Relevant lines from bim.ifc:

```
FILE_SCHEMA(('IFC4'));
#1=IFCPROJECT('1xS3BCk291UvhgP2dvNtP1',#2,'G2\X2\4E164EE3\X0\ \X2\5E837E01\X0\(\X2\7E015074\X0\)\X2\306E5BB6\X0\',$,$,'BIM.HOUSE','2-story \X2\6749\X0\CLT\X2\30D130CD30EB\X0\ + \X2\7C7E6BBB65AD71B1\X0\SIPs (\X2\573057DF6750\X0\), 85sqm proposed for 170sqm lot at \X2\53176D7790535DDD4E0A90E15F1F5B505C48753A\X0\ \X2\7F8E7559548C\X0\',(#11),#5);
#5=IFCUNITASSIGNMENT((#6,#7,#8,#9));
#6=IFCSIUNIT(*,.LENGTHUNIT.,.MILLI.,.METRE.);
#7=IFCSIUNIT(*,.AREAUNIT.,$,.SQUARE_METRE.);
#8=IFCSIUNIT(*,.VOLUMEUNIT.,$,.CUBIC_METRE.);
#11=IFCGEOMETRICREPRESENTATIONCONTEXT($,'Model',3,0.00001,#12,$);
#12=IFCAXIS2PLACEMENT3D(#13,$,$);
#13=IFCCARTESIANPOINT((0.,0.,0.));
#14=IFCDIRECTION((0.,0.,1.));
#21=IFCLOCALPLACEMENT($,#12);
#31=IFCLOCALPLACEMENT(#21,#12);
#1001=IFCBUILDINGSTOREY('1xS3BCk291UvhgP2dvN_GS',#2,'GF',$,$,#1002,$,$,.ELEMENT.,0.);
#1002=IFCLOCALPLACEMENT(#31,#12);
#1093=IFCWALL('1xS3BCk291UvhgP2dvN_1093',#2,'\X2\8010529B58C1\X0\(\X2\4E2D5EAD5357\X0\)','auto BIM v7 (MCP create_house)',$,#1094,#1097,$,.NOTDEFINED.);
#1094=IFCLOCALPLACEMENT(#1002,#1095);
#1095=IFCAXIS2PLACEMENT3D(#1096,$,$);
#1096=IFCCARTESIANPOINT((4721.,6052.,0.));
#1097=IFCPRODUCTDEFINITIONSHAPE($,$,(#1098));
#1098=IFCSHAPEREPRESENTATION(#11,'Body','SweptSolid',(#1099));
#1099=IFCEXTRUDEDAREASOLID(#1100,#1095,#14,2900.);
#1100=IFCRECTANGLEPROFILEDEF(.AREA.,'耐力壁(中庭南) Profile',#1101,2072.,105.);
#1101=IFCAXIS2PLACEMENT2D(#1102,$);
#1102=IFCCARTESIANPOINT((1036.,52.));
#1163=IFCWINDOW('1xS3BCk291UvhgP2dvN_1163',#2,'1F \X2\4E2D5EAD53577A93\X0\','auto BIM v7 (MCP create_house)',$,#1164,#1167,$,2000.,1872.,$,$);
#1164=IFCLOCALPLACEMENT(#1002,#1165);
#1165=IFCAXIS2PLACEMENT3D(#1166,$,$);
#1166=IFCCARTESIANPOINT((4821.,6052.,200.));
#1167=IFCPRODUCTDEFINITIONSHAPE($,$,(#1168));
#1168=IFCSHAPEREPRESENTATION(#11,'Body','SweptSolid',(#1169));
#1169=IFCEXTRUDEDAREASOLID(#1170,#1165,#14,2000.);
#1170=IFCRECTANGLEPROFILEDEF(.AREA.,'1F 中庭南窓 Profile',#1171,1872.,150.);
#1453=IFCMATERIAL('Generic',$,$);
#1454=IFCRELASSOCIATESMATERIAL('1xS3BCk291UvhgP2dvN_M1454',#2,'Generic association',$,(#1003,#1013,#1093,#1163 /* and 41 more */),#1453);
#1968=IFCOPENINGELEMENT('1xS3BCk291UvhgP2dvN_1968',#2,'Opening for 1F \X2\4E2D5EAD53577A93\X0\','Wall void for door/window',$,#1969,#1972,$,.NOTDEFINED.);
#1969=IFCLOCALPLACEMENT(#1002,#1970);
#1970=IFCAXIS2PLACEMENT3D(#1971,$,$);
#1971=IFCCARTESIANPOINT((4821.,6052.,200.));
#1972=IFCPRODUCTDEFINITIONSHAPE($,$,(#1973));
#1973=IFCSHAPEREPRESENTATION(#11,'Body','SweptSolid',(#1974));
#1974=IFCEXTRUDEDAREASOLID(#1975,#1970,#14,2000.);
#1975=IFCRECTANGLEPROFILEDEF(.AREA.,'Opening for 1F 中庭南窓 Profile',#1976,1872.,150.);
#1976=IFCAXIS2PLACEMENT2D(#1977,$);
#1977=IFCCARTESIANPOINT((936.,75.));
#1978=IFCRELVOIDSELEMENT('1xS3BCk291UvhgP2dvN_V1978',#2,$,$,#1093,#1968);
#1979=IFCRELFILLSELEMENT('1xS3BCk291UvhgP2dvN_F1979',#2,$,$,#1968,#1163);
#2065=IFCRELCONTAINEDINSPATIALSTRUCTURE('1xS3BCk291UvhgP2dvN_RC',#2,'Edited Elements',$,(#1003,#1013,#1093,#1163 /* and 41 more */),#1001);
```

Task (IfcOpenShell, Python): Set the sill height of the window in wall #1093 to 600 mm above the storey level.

```python
import numpy as np
import ifcopenshell
import ifcopenshell.api.geometry
import ifcopenshell.geom
import ifcopenshell.util.element
import ifcopenshell.util.placement
import ifcopenshell.util.shape
import ifcopenshell.util.unit

model = ifcopenshell.open("bim.ifc")
unit_scale = ifcopenshell.util.unit.calculate_unit_scale(model)

window = model.by_guid("1xS3BCk291UvhgP2dvN_1163")
opening = window.FillsVoids[0].RelatingOpeningElement
storey = ifcopenshell.util.element.get_container(window, ifc_class="IfcBuildingStorey")
level = ifcopenshell.util.placement.get_local_placement(storey.ObjectPlacement)[2, 3]

# The opening's origin need not be at the sill, so measure its lowest point.
shape = ifcopenshell.geom.create_shape(ifcopenshell.geom.settings(), opening)
bottom = ifcopenshell.util.shape.get_shape_bottom_elevation(shape, shape.geometry) / unit_scale
dz = level + 0.6 / unit_scale - bottom

shift = np.array([0.0, 0.0, dz])
# The window is not placed relative to its opening, so move both.
for product in (opening, window):
    matrix = ifcopenshell.util.placement.get_local_placement(product.ObjectPlacement)
    matrix[:3, 3] += shift
    ifcopenshell.api.geometry.edit_object_placement(model, product=product, matrix=matrix, is_si=False)

print(f"moved by {dz * unit_scale:+.3f} m")

model.write("bim-out.ifc")
```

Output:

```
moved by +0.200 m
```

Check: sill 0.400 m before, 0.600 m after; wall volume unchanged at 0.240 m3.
